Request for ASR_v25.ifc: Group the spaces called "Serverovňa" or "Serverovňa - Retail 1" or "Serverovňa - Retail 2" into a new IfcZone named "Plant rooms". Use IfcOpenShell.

First a look at what the model holds.

```python
import ifcopenshell

model = ifcopenshell.open("ASR_v25.ifc")
print(model.schema)
seen = {}
for space in model.by_type("IfcSpace"):
    seen[space.LongName] = seen.get(space.LongName, 0) + 1
for name, count in sorted(seen.items(), key=str):
    print(count, "x", name)
print("zones:", [z.Name for z in model.by_type("IfcZone")][:20])
```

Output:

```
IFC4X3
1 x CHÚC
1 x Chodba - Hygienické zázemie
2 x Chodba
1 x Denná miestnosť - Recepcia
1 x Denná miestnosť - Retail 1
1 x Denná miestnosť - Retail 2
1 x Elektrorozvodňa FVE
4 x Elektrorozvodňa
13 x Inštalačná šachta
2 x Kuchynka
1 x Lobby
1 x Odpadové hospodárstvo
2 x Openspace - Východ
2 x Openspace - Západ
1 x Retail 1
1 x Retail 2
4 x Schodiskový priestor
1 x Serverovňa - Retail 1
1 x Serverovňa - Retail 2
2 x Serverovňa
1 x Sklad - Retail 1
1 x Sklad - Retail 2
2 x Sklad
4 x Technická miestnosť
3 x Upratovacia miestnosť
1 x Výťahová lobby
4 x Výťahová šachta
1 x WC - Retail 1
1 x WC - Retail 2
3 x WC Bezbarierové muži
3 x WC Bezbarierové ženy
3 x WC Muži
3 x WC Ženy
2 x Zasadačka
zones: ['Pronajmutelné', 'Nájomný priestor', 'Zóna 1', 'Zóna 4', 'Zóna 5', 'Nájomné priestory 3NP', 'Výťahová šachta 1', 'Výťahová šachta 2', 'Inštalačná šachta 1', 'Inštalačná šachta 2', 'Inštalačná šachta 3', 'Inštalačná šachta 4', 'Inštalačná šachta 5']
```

```python
import ifcopenshell
import ifcopenshell.api.group
import ifcopenshell.api.root

model = ifcopenshell.open("ASR_v25.ifc")

names = {"Serverovňa", "Serverovňa - Retail 1", "Serverovňa - Retail 2"}
spaces = [s for s in model.by_type("IfcSpace") if s.LongName in names]

zone = ifcopenshell.api.root.create_entity(model, ifc_class="IfcZone", name="Plant rooms")
ifcopenshell.api.group.assign_group(model, products=spaces, group=zone)
print(len(spaces), "spaces in", zone.Name)

model.write("ASR_v25_edited.ifc")
```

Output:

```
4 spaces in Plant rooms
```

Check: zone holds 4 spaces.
